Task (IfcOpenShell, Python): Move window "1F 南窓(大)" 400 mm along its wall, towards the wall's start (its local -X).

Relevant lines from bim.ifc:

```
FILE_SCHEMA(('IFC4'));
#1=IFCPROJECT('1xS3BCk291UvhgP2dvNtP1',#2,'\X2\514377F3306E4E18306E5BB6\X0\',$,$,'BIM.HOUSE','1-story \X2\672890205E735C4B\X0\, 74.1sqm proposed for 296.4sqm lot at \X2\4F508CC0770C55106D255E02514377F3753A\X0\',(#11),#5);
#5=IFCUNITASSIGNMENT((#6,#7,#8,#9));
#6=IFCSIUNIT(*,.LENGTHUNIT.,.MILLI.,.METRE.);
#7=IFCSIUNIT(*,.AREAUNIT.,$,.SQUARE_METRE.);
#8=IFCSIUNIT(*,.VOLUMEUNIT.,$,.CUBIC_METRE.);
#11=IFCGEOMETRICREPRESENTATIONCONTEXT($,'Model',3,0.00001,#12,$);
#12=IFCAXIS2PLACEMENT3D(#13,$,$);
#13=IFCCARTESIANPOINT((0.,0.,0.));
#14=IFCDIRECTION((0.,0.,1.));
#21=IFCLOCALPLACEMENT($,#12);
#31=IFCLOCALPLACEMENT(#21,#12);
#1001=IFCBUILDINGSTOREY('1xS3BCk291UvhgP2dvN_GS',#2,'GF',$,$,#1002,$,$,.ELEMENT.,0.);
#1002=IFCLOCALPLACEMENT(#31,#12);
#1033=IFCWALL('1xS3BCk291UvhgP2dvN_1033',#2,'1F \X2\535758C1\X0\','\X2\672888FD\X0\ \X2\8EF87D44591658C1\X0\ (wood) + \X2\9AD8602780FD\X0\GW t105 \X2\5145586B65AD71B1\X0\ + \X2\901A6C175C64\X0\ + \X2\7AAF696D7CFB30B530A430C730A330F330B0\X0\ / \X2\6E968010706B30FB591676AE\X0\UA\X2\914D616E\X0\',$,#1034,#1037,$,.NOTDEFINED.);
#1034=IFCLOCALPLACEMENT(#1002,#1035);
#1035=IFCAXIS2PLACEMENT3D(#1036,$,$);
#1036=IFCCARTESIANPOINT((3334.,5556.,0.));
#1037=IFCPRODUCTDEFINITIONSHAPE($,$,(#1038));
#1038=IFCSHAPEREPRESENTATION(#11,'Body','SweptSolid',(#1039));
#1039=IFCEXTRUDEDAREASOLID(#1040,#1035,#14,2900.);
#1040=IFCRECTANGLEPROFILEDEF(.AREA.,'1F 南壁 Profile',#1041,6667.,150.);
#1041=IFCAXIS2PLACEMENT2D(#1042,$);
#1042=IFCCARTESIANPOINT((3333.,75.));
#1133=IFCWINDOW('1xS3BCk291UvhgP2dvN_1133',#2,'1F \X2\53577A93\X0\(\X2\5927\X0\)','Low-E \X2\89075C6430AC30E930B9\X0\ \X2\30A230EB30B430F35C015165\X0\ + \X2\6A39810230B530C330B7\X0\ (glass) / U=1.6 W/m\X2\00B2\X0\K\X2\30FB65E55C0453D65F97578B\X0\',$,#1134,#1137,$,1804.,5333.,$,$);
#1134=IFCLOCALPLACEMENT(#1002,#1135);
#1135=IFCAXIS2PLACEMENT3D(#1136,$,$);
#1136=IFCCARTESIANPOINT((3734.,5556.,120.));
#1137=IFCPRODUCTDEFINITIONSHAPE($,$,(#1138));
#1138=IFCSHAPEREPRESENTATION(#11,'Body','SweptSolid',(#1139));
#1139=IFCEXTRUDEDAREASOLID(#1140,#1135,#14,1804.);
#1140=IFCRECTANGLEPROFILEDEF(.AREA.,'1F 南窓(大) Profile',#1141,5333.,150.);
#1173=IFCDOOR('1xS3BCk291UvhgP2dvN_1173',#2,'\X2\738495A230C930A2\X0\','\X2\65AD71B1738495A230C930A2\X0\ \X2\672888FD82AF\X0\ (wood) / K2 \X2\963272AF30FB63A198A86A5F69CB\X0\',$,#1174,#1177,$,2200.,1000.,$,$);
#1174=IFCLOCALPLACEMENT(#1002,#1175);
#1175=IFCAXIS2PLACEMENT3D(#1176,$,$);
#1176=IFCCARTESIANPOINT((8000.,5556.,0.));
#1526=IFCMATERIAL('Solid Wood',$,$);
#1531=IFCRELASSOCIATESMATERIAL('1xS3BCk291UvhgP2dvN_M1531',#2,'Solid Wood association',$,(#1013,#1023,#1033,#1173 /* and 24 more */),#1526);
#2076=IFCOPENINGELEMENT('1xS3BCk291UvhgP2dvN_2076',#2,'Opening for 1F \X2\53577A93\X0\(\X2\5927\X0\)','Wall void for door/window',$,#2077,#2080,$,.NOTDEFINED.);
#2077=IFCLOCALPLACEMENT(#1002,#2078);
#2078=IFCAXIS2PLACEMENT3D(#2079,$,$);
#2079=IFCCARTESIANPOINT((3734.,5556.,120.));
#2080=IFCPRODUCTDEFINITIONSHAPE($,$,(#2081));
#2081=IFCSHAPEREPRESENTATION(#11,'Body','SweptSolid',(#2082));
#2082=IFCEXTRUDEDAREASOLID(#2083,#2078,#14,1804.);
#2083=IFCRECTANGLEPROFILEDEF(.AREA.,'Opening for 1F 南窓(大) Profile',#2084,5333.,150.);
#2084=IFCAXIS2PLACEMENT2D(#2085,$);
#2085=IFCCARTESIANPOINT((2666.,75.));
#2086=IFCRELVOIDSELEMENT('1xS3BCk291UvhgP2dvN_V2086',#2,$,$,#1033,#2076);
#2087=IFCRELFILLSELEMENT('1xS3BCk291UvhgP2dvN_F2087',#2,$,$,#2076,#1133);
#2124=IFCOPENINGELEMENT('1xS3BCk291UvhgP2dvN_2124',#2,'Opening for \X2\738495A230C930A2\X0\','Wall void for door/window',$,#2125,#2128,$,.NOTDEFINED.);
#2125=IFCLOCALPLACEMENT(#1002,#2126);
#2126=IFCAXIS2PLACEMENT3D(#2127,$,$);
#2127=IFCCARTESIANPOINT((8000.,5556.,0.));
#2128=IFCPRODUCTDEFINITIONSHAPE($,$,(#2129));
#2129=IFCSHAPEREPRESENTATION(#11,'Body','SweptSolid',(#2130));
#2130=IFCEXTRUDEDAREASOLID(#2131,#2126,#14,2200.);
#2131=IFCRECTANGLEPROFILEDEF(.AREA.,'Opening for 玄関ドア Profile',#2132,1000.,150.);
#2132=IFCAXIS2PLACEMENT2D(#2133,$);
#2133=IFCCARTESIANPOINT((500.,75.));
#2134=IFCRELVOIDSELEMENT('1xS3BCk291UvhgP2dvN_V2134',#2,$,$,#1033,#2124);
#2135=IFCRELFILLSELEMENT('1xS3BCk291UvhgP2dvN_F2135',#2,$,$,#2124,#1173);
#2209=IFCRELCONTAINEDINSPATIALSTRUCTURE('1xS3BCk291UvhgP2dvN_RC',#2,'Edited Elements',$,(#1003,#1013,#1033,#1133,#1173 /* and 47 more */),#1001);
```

```python
import ifcopenshell
import ifcopenshell.api.geometry
import ifcopenshell.util.placement

model = ifcopenshell.open("bim.ifc")

window = model.by_id(1133)
opening = window.FillsVoids[0].RelatingOpeningElement
wall = opening.VoidsElements[0].RelatingBuildingElement

wall_matrix = ifcopenshell.util.placement.get_local_placement(wall.ObjectPlacement)
shift = wall_matrix[:3, 0] * -400.0
before = ifcopenshell.util.placement.get_local_placement(window.ObjectPlacement)[:3, 3].copy()

# The window is not placed relative to its opening, so move both.
for product in (opening, window):
    matrix = ifcopenshell.util.placement.get_local_placement(product.ObjectPlacement)
    matrix[:3, 3] += shift
    ifcopenshell.api.geometry.edit_object_placement(model, product=product, matrix=matrix, is_si=False)

after = ifcopenshell.util.placement.get_local_placement(window.ObjectPlacement)[:3, 3]
print("window moved by", (after - before).round(3) + 0.0)

model.write("bim_v2.ifc")
```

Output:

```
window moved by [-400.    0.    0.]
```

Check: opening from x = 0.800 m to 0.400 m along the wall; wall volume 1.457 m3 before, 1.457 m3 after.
